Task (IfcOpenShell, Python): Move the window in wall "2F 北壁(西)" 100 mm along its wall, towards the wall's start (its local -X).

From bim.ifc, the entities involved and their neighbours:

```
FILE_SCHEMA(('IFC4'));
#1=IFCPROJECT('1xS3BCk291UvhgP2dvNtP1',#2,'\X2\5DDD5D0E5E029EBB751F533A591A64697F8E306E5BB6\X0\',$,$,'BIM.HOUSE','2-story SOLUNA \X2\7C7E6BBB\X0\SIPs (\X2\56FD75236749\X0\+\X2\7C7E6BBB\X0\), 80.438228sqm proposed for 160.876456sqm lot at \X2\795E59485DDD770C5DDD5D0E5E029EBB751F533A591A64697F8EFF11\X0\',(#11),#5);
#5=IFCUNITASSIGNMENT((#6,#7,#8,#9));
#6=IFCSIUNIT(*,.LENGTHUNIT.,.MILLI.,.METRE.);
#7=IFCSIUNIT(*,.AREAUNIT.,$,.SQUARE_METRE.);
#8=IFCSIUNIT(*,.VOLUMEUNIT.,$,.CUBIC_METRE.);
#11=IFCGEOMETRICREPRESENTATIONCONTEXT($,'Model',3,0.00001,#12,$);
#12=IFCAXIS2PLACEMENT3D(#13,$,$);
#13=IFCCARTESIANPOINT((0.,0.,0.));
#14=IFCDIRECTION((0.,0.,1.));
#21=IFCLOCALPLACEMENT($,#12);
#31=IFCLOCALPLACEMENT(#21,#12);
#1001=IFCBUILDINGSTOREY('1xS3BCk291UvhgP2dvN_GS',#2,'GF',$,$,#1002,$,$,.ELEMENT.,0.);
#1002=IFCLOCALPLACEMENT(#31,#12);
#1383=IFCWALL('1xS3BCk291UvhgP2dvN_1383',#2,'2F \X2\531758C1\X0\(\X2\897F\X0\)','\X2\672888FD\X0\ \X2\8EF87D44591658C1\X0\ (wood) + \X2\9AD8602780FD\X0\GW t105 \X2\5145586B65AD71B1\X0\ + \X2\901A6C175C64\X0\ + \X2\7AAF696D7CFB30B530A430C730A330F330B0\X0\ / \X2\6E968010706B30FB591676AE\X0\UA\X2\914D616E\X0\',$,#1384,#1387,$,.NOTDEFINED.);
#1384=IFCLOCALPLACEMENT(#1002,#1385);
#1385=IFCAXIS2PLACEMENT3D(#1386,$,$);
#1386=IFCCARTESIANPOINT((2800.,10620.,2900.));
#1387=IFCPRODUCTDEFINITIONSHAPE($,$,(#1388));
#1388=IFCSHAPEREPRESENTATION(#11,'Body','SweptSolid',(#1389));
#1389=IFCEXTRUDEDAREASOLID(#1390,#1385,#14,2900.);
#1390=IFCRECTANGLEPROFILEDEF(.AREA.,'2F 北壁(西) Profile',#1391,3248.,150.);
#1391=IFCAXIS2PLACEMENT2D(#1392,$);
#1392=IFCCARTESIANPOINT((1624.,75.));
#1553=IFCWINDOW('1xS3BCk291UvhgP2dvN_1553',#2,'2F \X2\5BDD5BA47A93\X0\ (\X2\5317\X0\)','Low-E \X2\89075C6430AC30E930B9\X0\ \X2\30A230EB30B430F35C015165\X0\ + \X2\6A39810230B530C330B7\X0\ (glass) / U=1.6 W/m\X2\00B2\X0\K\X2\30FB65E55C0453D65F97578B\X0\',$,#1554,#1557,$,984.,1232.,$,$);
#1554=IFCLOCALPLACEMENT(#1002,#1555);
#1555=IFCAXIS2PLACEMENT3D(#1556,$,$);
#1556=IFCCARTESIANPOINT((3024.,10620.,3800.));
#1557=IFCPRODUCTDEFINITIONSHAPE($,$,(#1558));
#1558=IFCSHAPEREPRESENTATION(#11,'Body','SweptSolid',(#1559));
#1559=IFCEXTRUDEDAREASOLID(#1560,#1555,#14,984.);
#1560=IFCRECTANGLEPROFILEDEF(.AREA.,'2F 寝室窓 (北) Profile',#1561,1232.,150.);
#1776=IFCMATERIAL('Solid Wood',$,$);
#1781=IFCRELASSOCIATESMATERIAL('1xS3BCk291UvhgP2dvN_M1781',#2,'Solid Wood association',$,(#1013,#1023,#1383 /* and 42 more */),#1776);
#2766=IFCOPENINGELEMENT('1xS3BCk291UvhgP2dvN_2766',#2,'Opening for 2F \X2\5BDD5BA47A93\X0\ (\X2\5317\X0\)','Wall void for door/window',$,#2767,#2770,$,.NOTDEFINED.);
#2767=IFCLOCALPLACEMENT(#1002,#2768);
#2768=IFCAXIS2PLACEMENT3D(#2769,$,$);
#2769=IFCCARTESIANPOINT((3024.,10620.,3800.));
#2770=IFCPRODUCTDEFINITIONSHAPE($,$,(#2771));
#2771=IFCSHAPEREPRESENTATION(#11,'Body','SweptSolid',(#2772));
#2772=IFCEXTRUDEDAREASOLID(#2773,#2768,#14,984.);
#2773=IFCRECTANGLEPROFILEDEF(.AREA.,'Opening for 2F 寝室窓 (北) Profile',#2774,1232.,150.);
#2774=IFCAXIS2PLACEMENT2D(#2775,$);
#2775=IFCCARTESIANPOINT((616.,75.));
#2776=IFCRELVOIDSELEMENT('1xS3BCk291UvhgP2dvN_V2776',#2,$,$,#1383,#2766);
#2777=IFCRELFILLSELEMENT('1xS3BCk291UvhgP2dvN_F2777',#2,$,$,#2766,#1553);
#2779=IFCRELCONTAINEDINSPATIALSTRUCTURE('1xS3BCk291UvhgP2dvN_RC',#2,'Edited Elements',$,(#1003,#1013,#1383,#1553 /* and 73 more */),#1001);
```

```python
import ifcopenshell
import ifcopenshell.api.geometry
import ifcopenshell.util.placement

model = ifcopenshell.open("bim.ifc")

window = model.by_id(1553)
opening = window.FillsVoids[0].RelatingOpeningElement
wall = opening.VoidsElements[0].RelatingBuildingElement

wall_matrix = ifcopenshell.util.placement.get_local_placement(wall.ObjectPlacement)
shift = wall_matrix[:3, 0] * -100.0
before = ifcopenshell.util.placement.get_local_placement(window.ObjectPlacement)[:3, 3].copy()

# The window is not placed relative to its opening, so move both.
for product in (opening, window):
    matrix = ifcopenshell.util.placement.get_local_placement(product.ObjectPlacement)
    matrix[:3, 3] += shift
    ifcopenshell.api.geometry.edit_object_placement(model, product=product, matrix=matrix, is_si=False)

after = ifcopenshell.util.placement.get_local_placement(window.ObjectPlacement)[:3, 3]
print("window moved by", (after - before).round(3) + 0.0)

model.write("bim_v2.ifc")
```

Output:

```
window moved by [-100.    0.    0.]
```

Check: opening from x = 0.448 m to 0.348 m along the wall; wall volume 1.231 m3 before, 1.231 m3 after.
